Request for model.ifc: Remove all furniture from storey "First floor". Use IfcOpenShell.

First a look at what the model holds.

```python
import ifcopenshell
import ifcopenshell.util.element

model = ifcopenshell.open("model.ifc")
print(model.schema)
storey = next(s for s in model.by_type("IfcBuildingStorey") if s.Name == "First floor")
furniture = [e for e in ifcopenshell.util.element.get_decomposition(storey) if e.is_a("IfcFurnishingElement")]
seen = {}
for e in furniture:
    element_type = ifcopenshell.util.element.get_type(e)
    name = element_type.Name if element_type not in (None, e) else None
    seen[name] = seen.get(name, 0) + 1
for name, count in sorted(seen.items(), key=str):
    print(count, "x", name)
```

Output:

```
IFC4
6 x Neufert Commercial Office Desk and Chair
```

```python
import ifcopenshell
import ifcopenshell.api.root
import ifcopenshell.util.element

model = ifcopenshell.open("model.ifc")

storey = next(s for s in model.by_type("IfcBuildingStorey") if s.Name == "First floor")
furniture = [e for e in ifcopenshell.util.element.get_decomposition(storey) if e.is_a("IfcFurnishingElement")]

for e in furniture:
    ifcopenshell.api.root.remove_product(model, product=e)
print(len(furniture), "removed")

model.write("model_rev.ifc")
```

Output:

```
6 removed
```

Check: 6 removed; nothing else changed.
